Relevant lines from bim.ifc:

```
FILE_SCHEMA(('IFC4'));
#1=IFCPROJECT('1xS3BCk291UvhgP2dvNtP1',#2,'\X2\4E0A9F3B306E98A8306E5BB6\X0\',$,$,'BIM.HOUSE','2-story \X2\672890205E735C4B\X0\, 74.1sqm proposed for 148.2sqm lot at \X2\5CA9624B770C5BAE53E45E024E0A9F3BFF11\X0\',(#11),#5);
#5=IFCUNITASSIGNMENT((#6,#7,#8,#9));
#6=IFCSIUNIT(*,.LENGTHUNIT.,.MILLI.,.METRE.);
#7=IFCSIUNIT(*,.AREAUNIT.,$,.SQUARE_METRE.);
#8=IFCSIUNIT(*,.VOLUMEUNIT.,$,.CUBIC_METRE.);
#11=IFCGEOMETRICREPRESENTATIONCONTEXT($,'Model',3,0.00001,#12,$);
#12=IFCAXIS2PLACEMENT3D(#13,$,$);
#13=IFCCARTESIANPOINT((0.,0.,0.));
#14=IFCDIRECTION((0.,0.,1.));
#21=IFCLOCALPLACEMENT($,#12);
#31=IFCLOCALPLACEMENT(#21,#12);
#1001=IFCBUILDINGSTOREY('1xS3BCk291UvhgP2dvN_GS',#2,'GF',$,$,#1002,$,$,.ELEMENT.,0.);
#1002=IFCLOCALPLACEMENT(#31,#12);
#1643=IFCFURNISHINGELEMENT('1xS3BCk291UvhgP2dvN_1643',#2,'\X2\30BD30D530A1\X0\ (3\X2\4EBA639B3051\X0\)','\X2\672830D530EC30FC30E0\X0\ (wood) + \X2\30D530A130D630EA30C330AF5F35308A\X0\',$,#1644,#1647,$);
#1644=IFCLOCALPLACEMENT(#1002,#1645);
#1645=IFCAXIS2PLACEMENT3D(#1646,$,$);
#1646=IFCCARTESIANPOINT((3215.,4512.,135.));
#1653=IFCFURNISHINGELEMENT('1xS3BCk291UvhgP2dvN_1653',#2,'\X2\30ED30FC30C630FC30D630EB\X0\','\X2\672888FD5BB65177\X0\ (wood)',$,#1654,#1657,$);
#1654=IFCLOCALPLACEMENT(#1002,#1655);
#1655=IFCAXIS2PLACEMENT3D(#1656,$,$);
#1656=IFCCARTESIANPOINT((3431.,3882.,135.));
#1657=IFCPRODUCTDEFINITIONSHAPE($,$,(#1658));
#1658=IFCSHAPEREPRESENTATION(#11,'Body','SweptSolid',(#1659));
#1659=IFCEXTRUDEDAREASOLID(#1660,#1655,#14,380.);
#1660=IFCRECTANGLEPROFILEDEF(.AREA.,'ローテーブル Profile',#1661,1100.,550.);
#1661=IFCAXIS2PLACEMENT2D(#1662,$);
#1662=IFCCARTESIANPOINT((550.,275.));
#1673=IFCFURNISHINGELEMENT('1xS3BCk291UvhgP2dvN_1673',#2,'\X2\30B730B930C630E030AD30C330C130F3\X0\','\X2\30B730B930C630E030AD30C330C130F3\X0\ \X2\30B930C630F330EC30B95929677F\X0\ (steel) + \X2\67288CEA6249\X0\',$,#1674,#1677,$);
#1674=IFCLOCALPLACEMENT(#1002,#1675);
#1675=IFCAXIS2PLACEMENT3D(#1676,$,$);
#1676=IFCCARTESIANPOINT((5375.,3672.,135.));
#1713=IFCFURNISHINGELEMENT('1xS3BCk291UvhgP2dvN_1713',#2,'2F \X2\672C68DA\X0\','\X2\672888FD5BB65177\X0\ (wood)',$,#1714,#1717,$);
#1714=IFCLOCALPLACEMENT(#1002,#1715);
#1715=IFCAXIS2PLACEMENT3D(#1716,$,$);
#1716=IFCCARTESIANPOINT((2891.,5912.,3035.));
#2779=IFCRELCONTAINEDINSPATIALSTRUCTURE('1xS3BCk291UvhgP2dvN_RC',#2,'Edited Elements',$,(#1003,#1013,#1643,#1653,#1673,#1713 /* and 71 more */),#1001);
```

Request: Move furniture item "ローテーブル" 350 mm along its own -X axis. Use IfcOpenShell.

```python
import ifcopenshell
import ifcopenshell.api.geometry
import ifcopenshell.util.placement

model = ifcopenshell.open("bim.ifc")

item = model.by_guid("1xS3BCk291UvhgP2dvN_1653")
matrix = ifcopenshell.util.placement.get_local_placement(item.ObjectPlacement)
matrix[:3, 3] -= matrix[:3, 0] * 350.0
ifcopenshell.api.geometry.edit_object_placement(model, product=item, matrix=matrix, is_si=False)

print(ifcopenshell.util.placement.get_local_placement(item.ObjectPlacement).round(3) + 0.0)

model.write("bim_updated.ifc")
```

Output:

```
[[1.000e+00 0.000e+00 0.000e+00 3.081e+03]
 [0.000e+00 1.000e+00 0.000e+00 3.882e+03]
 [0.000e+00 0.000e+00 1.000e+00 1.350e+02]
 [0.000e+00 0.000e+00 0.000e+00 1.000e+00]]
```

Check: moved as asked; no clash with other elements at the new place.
